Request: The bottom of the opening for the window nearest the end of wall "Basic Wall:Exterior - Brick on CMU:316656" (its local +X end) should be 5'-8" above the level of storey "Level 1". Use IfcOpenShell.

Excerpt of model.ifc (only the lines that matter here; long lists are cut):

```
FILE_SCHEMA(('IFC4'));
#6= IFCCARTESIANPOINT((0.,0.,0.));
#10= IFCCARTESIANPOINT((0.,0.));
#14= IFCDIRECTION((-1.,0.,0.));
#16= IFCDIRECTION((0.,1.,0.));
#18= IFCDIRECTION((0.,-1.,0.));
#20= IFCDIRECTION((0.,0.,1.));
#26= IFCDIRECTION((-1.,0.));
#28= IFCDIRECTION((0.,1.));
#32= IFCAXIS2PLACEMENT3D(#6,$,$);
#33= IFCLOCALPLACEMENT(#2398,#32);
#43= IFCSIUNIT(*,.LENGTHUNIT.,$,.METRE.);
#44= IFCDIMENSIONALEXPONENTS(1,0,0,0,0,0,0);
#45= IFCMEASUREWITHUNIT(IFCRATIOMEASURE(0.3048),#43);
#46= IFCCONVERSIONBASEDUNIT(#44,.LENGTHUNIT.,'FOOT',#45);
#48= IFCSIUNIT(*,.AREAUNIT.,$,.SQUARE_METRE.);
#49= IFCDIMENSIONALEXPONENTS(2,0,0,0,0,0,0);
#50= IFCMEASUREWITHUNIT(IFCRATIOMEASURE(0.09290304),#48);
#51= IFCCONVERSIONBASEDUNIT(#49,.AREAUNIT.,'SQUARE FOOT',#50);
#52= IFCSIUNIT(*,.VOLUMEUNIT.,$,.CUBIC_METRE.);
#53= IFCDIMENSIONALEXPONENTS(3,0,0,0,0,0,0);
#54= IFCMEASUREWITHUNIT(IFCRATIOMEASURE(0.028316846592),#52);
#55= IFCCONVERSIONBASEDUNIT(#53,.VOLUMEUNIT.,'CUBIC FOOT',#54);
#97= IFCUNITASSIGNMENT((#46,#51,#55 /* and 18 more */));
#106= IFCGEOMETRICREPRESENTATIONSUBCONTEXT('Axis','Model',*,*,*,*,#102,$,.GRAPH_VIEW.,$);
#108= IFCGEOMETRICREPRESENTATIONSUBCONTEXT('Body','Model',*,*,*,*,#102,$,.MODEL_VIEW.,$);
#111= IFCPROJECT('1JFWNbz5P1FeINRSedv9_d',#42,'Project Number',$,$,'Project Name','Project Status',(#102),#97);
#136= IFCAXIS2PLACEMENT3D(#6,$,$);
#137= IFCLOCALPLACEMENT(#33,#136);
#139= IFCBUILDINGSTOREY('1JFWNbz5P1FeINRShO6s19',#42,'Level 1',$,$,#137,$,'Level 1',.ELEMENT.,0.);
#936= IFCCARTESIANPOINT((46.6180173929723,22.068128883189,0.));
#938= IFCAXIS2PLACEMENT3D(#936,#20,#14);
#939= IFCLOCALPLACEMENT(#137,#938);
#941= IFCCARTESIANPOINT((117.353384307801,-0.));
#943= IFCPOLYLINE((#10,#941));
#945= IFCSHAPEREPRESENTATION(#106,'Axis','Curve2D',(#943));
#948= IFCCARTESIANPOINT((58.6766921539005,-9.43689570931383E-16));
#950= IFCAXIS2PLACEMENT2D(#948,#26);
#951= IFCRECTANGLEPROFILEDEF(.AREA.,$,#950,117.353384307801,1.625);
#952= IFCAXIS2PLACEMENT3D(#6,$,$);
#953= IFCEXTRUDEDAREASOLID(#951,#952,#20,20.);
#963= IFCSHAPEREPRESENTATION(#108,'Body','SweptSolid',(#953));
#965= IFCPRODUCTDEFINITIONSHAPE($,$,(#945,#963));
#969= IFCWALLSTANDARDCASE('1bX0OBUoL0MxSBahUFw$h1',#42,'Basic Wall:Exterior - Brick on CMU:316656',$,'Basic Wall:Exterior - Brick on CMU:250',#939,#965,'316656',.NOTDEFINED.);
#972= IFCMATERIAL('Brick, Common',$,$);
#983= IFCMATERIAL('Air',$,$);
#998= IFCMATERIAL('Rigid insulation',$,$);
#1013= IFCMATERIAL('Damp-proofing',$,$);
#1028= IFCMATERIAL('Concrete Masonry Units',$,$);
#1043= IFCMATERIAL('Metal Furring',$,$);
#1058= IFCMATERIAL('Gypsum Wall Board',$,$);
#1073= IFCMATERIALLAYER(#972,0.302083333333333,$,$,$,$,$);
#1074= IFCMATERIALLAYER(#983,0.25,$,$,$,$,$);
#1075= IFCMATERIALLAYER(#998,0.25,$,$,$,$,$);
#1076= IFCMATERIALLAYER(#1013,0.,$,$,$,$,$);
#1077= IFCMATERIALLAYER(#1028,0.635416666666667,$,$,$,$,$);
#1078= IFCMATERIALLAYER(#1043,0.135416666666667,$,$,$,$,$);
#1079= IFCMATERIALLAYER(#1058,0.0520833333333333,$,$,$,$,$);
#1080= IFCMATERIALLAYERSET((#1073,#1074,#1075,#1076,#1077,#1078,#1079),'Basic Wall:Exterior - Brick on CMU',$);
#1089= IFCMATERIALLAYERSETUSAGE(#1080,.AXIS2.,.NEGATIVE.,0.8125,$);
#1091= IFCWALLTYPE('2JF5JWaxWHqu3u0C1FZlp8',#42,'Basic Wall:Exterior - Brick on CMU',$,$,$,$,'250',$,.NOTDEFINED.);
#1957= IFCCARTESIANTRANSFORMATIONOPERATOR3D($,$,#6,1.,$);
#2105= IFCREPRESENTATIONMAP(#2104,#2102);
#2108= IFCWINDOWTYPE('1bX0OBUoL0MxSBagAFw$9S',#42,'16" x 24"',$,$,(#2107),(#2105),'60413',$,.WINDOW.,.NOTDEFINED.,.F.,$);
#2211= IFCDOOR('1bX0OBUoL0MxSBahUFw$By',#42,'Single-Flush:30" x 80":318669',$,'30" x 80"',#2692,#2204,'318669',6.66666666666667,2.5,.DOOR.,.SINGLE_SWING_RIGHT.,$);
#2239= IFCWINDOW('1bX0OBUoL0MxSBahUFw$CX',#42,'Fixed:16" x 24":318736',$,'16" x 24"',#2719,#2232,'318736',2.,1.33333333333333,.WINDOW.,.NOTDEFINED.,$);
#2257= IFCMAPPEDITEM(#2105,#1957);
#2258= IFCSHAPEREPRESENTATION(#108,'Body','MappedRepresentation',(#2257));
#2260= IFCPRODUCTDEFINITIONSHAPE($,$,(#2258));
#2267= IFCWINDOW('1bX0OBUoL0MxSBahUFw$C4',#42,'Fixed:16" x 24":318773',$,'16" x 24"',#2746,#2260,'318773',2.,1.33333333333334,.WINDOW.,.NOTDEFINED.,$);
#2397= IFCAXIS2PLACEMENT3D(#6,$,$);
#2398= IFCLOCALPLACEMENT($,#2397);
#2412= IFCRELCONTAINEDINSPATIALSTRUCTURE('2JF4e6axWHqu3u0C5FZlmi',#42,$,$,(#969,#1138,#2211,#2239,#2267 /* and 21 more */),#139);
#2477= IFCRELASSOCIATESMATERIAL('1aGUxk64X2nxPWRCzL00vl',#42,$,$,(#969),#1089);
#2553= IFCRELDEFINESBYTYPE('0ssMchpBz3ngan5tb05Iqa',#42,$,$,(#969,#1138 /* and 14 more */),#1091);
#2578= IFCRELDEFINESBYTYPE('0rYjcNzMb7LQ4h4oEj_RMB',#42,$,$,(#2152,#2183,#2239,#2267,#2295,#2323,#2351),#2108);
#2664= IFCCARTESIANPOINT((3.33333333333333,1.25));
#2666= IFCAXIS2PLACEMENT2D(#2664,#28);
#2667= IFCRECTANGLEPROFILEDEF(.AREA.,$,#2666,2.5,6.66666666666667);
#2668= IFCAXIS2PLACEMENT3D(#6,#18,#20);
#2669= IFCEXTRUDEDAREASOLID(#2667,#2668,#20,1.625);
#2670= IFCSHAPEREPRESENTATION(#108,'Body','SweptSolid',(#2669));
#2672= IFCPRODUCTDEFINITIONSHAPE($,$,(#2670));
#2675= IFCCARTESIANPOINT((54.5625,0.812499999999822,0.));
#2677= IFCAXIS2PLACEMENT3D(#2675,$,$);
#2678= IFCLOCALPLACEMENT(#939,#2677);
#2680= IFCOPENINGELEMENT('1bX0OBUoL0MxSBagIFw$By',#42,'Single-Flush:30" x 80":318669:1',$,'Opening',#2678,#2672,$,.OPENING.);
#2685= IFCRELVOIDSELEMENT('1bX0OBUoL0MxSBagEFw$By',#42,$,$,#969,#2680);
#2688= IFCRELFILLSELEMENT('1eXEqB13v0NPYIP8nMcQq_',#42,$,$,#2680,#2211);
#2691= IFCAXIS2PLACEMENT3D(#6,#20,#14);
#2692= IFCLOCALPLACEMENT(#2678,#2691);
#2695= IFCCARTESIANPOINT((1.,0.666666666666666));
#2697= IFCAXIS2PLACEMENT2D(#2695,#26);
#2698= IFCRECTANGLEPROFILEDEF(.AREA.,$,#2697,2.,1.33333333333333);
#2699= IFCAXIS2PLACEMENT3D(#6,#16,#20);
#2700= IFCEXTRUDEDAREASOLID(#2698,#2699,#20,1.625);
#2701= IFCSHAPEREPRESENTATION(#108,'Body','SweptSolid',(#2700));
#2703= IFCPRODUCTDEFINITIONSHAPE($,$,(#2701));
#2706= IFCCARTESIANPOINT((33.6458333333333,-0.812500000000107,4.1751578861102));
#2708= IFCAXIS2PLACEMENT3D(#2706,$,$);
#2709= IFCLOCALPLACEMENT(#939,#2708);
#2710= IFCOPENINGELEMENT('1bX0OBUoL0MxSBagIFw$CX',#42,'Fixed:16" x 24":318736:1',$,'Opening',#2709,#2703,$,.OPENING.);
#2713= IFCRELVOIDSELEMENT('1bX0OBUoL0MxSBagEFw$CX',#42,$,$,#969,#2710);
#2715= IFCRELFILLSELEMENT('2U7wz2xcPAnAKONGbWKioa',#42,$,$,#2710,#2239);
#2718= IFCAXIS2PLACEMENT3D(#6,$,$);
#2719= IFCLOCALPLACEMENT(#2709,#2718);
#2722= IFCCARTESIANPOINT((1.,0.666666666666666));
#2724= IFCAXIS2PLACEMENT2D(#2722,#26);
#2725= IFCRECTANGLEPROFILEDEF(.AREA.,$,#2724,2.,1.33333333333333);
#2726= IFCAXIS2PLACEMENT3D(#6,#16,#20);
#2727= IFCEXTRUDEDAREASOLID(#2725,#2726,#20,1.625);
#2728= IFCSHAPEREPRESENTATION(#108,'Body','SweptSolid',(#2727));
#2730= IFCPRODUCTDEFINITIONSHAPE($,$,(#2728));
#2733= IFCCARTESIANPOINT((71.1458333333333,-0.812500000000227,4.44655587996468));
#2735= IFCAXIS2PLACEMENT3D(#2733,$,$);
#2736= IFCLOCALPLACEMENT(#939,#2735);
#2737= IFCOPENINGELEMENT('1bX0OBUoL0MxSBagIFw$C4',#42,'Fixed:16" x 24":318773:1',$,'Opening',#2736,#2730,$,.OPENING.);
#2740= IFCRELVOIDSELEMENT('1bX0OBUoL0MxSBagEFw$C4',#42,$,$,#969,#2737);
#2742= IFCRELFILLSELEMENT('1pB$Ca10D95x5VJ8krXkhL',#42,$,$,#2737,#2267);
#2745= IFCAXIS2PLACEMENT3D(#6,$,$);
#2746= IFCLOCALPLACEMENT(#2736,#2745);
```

```python
import numpy as np
import ifcopenshell
import ifcopenshell.api.geometry
import ifcopenshell.geom
import ifcopenshell.util.element
import ifcopenshell.util.placement
import ifcopenshell.util.shape
import ifcopenshell.util.unit

model = ifcopenshell.open("model.ifc")
unit_scale = ifcopenshell.util.unit.calculate_unit_scale(model)

window = model.by_guid("1bX0OBUoL0MxSBahUFw$C4")
opening = window.FillsVoids[0].RelatingOpeningElement
storey = ifcopenshell.util.element.get_container(window, ifc_class="IfcBuildingStorey")
level = ifcopenshell.util.placement.get_local_placement(storey.ObjectPlacement)[2, 3]

# The opening's origin need not be at the sill, so measure its lowest point.
shape = ifcopenshell.geom.create_shape(ifcopenshell.geom.settings(), opening)
bottom = ifcopenshell.util.shape.get_shape_bottom_elevation(shape, shape.geometry) / unit_scale
dz = level + 68 * 0.0254 / unit_scale - bottom

shift = np.array([0.0, 0.0, dz])
# The window is placed relative to its opening, so it follows when the opening moves.
matrix = ifcopenshell.util.placement.get_local_placement(opening.ObjectPlacement)
matrix[:3, 3] += shift
ifcopenshell.api.geometry.edit_object_placement(
    model, product=opening, matrix=matrix, is_si=False, should_transform_children=True
)

print(f"moved by {dz * unit_scale:+.3f} m")

model.write("model_v2.ifc")
```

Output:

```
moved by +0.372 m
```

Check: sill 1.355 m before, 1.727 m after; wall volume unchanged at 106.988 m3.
